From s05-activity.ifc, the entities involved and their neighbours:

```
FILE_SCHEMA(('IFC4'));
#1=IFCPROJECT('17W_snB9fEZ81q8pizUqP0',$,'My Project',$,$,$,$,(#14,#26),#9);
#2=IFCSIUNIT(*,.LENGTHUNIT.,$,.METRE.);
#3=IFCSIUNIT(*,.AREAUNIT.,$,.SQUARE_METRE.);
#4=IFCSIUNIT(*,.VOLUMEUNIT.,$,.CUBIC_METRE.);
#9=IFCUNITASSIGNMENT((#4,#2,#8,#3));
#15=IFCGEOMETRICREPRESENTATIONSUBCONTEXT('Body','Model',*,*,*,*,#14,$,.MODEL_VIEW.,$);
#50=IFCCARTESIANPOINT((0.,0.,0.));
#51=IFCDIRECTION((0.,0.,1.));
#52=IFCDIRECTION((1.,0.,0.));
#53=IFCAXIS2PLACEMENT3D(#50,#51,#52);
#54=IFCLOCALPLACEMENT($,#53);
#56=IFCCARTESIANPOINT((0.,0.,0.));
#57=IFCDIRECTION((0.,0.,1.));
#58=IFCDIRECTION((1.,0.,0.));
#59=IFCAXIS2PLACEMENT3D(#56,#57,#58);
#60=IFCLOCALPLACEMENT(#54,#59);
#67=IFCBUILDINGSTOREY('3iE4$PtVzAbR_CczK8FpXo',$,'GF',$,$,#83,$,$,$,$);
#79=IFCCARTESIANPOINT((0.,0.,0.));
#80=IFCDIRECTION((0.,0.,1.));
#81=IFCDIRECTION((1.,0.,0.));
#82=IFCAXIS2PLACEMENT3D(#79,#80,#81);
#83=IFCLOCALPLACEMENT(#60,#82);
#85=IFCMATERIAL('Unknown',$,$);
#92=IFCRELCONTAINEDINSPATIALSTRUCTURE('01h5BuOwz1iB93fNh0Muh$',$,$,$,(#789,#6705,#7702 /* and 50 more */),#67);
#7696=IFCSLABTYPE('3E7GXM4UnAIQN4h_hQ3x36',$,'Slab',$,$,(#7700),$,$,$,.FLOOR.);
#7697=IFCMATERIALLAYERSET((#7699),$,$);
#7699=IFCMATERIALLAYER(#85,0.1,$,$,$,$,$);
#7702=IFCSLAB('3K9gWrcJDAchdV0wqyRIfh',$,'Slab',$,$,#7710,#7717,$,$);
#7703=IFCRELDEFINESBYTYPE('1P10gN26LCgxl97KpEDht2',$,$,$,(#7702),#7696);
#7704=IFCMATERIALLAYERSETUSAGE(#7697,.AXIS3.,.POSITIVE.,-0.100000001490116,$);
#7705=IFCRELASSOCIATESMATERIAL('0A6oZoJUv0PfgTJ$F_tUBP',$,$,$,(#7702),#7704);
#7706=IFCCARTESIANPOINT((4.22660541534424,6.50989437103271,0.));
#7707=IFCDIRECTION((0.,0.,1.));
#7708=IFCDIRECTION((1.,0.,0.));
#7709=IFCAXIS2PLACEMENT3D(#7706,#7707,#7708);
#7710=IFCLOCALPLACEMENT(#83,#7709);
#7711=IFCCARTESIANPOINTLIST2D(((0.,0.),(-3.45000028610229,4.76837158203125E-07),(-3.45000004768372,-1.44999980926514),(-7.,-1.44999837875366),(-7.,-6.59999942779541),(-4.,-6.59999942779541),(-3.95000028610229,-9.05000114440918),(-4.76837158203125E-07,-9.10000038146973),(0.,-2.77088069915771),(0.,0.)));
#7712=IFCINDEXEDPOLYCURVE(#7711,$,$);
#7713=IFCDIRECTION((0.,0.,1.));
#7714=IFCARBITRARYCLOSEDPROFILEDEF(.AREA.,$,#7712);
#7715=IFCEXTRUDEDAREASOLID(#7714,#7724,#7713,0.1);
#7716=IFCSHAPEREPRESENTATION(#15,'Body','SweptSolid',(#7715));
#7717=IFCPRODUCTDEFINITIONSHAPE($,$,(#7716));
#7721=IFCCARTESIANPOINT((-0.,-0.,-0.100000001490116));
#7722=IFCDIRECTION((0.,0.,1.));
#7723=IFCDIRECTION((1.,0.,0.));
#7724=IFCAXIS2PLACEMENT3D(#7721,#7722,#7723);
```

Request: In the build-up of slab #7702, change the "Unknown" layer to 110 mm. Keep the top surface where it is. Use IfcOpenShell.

```python
import ifcopenshell
import ifcopenshell.util.element
import ifcopenshell.util.representation

model = ifcopenshell.open("s05-activity.ifc")

layer_set = model.by_id(7697)
layer = next(l for l in layer_set.MaterialLayers if l.Material and l.Material.Name == "Unknown")
change = 0.11 - layer.LayerThickness
layer.LayerThickness += change

# Geometry does not follow the layer set by itself.
slabs = [e for e in ifcopenshell.util.element.get_elements_by_material(model, layer_set) if e.is_a("IfcSlab")]
for slab in sorted(slabs, key=lambda e: e.id()):
    body = ifcopenshell.util.representation.get_representation(slab, "Model", "Body")
    solid = body.Items[0]
    old_depth = solid.Depth
    solid.Depth += change
    # Extruded upwards: lower the start of the extrusion so the top stays.
    x, y, z = solid.Position.Location.Coordinates
    solid.Position.Location = model.createIfcCartesianPoint((x, y, z - change))
    print(slab.id(), f"{old_depth:g} -> {solid.Depth:g}")

# The layers are counted up from the underside, which has moved.
for usage in {ifcopenshell.util.element.get_material(slab) for slab in slabs}:
    usage.OffsetFromReferenceLine -= change

model.write("s05-activity_edited.ifc")
```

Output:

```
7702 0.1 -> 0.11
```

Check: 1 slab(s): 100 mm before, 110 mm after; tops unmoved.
